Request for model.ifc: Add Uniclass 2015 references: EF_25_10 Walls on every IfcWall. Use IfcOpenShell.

First a look at what the model holds.

```python
import ifcopenshell

model = ifcopenshell.open("model.ifc")
print(model.schema)
print("classifications:", [c.Name for c in model.by_type("IfcClassification")])
for ifc_class in ("IfcDoor", "IfcRoof", "IfcStair", "IfcWall", "IfcWindow"):
    print(ifc_class, len(model.by_type(ifc_class)))
```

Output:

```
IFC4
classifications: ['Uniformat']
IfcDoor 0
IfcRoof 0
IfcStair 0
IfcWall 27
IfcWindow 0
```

```python
import ifcopenshell
import ifcopenshell.api.classification

model = ifcopenshell.open("model.ifc")

system = ifcopenshell.api.classification.add_classification(model, classification="Uniclass 2015")

codes = {
    "IfcWall": ("EF_25_10", "Walls"),
}
for ifc_class, (code, name) in codes.items():
    products = model.by_type(ifc_class)
    ifcopenshell.api.classification.add_reference(
        model, products=products, classification=system, identification=code, name=name
    )
    print(code, len(products))

model.write("model_updated.ifc")
```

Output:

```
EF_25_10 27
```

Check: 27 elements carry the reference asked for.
